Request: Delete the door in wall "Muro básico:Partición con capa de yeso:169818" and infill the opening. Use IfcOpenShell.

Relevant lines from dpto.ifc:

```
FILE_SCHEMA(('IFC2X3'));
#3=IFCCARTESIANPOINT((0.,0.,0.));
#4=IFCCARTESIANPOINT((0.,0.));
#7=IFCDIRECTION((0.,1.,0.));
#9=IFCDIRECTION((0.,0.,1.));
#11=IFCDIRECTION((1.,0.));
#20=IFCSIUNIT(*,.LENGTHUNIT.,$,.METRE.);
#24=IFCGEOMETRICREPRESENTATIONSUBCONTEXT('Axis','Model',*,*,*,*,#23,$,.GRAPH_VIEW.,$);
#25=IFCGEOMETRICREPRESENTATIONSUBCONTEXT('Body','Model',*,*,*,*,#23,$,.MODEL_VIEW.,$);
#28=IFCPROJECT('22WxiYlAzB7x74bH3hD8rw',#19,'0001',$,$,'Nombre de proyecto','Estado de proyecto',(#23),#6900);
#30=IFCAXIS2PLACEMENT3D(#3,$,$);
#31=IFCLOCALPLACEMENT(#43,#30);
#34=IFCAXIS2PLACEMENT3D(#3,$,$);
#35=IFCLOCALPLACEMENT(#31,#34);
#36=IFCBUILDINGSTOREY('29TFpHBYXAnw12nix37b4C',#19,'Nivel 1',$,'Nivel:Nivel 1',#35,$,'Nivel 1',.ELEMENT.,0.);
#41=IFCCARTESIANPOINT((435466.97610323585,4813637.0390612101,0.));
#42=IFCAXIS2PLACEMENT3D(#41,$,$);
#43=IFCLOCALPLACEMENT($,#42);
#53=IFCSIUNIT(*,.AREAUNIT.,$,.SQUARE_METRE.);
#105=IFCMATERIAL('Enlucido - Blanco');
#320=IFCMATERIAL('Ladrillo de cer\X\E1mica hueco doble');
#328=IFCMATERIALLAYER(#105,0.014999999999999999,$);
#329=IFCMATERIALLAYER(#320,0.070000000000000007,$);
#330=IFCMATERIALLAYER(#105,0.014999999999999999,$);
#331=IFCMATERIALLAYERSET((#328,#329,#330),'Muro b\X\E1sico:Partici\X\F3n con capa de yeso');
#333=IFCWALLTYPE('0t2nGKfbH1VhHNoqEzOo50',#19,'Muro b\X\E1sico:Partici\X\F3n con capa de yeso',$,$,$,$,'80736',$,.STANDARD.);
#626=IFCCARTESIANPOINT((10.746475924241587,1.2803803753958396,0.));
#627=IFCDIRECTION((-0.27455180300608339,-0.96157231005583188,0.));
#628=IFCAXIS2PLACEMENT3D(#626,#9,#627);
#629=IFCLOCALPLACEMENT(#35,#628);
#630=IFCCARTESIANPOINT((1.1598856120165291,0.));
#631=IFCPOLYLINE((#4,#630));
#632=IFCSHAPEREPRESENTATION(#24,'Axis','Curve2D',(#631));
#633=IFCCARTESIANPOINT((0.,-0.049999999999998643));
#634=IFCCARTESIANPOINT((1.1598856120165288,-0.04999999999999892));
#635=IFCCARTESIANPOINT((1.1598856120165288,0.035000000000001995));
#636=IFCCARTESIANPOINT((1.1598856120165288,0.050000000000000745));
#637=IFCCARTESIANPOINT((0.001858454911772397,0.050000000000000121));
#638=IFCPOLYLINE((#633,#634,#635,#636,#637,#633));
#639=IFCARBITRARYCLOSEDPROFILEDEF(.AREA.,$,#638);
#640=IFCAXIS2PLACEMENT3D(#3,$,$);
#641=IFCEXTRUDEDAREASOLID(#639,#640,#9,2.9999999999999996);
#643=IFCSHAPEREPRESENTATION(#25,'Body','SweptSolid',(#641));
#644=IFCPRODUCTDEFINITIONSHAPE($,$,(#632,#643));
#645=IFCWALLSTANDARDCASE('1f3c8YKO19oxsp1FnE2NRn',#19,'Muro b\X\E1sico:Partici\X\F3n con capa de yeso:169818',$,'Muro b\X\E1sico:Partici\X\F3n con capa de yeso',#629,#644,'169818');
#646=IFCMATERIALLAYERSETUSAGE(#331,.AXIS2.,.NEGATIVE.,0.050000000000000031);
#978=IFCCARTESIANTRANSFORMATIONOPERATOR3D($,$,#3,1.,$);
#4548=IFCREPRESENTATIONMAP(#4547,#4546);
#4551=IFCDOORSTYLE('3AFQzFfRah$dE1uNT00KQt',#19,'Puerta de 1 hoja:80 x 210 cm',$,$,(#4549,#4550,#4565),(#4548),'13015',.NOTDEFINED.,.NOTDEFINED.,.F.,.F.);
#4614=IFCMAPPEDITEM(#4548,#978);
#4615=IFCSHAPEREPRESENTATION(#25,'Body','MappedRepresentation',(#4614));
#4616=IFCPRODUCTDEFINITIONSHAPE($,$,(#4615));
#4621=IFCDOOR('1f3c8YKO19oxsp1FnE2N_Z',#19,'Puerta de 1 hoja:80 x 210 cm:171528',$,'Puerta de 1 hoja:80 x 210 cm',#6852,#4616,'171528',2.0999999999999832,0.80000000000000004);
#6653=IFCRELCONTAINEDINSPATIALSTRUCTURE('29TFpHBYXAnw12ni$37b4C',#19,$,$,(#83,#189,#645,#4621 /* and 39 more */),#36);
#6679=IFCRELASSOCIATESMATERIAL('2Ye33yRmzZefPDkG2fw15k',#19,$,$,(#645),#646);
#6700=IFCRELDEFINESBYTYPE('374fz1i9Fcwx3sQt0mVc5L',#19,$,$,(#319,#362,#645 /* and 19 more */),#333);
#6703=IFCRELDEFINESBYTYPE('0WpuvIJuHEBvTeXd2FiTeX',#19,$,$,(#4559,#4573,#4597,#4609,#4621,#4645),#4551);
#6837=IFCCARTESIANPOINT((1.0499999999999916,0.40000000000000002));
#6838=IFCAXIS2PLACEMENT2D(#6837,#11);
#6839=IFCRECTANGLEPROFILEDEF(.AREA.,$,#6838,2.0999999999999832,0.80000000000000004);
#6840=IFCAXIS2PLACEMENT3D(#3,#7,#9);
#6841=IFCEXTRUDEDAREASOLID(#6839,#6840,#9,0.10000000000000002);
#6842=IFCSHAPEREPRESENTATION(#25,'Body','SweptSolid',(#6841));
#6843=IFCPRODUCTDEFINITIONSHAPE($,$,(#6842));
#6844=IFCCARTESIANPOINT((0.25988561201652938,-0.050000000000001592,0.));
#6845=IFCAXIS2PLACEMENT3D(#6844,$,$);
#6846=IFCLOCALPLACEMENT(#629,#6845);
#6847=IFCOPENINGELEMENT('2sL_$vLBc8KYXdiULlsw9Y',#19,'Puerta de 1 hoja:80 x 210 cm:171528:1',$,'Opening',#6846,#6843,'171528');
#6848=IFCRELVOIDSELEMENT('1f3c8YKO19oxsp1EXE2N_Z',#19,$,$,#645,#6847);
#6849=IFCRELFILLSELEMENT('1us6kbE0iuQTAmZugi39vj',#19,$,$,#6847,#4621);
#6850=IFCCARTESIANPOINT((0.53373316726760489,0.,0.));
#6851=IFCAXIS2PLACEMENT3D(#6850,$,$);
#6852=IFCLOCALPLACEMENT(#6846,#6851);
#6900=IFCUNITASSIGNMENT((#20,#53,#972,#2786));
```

```python
import ifcopenshell
import ifcopenshell.api.feature
import ifcopenshell.api.root
import ifcopenshell.geom
import ifcopenshell.util.shape

model = ifcopenshell.open("dpto.ifc")
settings = ifcopenshell.geom.settings()


def volume(element):
    """Net volume in cubic metres, openings subtracted."""
    shape = ifcopenshell.geom.create_shape(settings, element)
    return ifcopenshell.util.shape.get_volume(shape.geometry)


door = model.by_guid("1f3c8YKO19oxsp1FnE2N_Z")
opening = door.FillsVoids[0].RelatingOpeningElement
wall = opening.VoidsElements[0].RelatingBuildingElement
before = volume(wall)

ifcopenshell.api.root.remove_product(model, product=door)
ifcopenshell.api.feature.remove_feature(model, feature=opening)

after = volume(wall)

print(f"wall volume {before:.3f} -> {after:.3f} m3")

model.write("dpto_rev.ifc")
```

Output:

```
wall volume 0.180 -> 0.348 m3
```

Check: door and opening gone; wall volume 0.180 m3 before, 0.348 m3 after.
